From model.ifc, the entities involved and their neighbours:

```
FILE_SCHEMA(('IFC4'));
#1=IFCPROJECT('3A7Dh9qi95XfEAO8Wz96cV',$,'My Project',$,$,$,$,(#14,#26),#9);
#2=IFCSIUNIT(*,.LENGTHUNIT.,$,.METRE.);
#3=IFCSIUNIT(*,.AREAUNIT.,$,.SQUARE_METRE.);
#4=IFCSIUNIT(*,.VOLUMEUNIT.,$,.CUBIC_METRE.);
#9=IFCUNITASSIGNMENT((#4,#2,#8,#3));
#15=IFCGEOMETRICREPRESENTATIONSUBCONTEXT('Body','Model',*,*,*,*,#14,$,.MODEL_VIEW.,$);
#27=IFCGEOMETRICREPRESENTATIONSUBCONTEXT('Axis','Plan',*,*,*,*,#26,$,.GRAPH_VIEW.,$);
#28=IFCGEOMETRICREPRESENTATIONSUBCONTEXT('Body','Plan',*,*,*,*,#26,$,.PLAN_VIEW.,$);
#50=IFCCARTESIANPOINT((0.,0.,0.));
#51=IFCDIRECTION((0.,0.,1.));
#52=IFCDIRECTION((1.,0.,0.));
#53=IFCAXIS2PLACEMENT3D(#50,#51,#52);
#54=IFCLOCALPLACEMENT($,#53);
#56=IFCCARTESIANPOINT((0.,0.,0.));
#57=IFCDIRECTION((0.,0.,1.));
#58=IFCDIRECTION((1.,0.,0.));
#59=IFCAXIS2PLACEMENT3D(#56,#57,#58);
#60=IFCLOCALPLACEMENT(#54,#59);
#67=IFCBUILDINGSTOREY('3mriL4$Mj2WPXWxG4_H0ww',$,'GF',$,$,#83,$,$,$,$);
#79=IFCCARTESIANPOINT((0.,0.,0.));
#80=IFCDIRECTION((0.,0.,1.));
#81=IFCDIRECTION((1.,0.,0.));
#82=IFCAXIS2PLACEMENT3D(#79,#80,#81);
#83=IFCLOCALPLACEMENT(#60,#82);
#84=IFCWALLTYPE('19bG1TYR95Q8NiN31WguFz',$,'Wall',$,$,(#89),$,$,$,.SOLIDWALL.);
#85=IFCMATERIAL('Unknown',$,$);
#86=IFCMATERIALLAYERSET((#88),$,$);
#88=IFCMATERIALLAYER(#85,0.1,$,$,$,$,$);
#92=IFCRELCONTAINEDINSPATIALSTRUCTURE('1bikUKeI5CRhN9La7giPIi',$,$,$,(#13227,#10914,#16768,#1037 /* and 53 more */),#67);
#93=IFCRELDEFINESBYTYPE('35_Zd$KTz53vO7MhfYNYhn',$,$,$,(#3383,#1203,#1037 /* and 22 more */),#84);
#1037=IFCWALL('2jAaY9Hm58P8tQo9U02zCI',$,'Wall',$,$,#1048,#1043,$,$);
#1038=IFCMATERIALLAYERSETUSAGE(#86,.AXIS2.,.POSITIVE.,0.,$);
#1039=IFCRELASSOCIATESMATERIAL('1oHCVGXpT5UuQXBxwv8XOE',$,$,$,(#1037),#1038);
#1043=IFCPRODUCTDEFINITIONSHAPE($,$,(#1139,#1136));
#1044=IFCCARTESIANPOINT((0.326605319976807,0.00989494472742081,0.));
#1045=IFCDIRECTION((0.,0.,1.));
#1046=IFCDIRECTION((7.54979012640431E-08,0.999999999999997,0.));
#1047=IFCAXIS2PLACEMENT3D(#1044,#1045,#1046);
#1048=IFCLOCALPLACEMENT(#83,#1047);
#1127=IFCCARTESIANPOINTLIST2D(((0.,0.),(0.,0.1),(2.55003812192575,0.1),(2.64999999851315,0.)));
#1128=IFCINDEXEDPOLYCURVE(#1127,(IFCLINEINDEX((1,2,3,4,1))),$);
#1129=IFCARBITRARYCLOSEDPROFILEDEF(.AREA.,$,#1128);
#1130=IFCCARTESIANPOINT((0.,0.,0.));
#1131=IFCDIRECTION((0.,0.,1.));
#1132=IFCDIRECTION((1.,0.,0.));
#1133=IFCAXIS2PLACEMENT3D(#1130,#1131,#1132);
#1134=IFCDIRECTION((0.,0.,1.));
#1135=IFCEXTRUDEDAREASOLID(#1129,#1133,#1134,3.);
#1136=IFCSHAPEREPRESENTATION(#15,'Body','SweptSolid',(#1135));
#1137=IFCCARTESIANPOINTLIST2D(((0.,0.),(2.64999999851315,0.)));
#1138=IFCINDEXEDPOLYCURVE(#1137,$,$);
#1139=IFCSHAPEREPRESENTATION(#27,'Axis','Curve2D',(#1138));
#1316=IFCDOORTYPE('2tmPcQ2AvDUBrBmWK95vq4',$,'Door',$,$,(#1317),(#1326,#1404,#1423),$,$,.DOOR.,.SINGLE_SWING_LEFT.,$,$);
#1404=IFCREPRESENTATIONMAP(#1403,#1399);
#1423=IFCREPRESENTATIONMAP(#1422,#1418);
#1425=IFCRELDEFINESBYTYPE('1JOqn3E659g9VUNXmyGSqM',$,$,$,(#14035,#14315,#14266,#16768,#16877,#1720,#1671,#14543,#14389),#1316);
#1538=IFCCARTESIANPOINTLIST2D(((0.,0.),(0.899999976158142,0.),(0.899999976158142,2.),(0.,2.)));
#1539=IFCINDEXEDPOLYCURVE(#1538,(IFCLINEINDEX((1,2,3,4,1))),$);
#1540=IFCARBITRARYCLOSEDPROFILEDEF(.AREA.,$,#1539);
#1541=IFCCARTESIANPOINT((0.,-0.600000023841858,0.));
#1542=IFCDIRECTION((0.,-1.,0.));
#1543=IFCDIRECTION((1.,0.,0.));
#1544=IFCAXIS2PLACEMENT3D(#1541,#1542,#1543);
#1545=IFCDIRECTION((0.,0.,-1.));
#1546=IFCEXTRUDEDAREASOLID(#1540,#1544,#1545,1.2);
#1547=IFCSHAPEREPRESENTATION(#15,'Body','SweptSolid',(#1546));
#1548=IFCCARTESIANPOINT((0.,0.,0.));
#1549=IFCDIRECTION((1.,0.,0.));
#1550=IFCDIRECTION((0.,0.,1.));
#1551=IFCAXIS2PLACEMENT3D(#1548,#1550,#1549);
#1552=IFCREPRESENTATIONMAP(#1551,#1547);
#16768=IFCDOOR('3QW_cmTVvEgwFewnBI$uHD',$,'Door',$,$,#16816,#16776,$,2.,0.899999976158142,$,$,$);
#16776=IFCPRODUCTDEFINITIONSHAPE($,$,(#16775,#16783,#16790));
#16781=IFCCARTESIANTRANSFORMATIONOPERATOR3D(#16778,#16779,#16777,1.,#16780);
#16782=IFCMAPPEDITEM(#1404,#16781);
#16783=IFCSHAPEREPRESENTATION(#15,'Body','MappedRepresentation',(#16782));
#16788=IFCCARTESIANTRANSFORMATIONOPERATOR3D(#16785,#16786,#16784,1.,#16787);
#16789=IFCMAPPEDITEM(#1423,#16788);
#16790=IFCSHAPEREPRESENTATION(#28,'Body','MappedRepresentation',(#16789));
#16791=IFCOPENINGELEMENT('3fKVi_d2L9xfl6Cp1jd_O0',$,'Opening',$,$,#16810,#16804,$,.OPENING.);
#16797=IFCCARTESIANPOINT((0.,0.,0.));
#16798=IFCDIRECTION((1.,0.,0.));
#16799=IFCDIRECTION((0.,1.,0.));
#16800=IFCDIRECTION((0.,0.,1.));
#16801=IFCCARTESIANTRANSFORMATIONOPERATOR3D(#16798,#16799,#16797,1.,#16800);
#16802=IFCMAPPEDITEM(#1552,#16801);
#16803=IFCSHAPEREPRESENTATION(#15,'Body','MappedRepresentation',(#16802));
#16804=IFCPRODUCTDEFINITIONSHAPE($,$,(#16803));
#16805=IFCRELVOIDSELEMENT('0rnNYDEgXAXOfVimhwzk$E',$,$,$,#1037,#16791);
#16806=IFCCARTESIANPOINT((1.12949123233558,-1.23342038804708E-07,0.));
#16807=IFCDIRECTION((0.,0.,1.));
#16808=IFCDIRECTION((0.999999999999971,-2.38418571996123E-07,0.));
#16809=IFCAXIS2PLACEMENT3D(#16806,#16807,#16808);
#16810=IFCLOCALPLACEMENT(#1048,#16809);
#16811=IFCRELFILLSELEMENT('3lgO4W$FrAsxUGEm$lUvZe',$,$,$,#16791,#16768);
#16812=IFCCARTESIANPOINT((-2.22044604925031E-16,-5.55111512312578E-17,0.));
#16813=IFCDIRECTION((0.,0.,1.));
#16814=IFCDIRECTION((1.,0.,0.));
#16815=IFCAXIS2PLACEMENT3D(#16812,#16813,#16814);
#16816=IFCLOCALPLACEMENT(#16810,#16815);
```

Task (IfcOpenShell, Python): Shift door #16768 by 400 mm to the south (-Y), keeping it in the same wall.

```python
import ifcopenshell
import ifcopenshell.api.geometry
import ifcopenshell.util.placement

model = ifcopenshell.open("model.ifc")

door = model.by_guid("3QW_cmTVvEgwFewnBI$uHD")
opening = door.FillsVoids[0].RelatingOpeningElement
wall = opening.VoidsElements[0].RelatingBuildingElement

wall_matrix = ifcopenshell.util.placement.get_local_placement(wall.ObjectPlacement)
shift = wall_matrix[:3, 0] * -0.4
before = ifcopenshell.util.placement.get_local_placement(door.ObjectPlacement)[:3, 3].copy()

# The door is placed relative to its opening, so it follows when the opening moves.
matrix = ifcopenshell.util.placement.get_local_placement(opening.ObjectPlacement)
matrix[:3, 3] += shift
ifcopenshell.api.geometry.edit_object_placement(
    model, product=opening, matrix=matrix, is_si=False, should_transform_children=True
)

after = ifcopenshell.util.placement.get_local_placement(door.ObjectPlacement)[:3, 3]
print("door moved by", (after - before).round(3) + 0.0)

model.write("model_updated.ifc")
```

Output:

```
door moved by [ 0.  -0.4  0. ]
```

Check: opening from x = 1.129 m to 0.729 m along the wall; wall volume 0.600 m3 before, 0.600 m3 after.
